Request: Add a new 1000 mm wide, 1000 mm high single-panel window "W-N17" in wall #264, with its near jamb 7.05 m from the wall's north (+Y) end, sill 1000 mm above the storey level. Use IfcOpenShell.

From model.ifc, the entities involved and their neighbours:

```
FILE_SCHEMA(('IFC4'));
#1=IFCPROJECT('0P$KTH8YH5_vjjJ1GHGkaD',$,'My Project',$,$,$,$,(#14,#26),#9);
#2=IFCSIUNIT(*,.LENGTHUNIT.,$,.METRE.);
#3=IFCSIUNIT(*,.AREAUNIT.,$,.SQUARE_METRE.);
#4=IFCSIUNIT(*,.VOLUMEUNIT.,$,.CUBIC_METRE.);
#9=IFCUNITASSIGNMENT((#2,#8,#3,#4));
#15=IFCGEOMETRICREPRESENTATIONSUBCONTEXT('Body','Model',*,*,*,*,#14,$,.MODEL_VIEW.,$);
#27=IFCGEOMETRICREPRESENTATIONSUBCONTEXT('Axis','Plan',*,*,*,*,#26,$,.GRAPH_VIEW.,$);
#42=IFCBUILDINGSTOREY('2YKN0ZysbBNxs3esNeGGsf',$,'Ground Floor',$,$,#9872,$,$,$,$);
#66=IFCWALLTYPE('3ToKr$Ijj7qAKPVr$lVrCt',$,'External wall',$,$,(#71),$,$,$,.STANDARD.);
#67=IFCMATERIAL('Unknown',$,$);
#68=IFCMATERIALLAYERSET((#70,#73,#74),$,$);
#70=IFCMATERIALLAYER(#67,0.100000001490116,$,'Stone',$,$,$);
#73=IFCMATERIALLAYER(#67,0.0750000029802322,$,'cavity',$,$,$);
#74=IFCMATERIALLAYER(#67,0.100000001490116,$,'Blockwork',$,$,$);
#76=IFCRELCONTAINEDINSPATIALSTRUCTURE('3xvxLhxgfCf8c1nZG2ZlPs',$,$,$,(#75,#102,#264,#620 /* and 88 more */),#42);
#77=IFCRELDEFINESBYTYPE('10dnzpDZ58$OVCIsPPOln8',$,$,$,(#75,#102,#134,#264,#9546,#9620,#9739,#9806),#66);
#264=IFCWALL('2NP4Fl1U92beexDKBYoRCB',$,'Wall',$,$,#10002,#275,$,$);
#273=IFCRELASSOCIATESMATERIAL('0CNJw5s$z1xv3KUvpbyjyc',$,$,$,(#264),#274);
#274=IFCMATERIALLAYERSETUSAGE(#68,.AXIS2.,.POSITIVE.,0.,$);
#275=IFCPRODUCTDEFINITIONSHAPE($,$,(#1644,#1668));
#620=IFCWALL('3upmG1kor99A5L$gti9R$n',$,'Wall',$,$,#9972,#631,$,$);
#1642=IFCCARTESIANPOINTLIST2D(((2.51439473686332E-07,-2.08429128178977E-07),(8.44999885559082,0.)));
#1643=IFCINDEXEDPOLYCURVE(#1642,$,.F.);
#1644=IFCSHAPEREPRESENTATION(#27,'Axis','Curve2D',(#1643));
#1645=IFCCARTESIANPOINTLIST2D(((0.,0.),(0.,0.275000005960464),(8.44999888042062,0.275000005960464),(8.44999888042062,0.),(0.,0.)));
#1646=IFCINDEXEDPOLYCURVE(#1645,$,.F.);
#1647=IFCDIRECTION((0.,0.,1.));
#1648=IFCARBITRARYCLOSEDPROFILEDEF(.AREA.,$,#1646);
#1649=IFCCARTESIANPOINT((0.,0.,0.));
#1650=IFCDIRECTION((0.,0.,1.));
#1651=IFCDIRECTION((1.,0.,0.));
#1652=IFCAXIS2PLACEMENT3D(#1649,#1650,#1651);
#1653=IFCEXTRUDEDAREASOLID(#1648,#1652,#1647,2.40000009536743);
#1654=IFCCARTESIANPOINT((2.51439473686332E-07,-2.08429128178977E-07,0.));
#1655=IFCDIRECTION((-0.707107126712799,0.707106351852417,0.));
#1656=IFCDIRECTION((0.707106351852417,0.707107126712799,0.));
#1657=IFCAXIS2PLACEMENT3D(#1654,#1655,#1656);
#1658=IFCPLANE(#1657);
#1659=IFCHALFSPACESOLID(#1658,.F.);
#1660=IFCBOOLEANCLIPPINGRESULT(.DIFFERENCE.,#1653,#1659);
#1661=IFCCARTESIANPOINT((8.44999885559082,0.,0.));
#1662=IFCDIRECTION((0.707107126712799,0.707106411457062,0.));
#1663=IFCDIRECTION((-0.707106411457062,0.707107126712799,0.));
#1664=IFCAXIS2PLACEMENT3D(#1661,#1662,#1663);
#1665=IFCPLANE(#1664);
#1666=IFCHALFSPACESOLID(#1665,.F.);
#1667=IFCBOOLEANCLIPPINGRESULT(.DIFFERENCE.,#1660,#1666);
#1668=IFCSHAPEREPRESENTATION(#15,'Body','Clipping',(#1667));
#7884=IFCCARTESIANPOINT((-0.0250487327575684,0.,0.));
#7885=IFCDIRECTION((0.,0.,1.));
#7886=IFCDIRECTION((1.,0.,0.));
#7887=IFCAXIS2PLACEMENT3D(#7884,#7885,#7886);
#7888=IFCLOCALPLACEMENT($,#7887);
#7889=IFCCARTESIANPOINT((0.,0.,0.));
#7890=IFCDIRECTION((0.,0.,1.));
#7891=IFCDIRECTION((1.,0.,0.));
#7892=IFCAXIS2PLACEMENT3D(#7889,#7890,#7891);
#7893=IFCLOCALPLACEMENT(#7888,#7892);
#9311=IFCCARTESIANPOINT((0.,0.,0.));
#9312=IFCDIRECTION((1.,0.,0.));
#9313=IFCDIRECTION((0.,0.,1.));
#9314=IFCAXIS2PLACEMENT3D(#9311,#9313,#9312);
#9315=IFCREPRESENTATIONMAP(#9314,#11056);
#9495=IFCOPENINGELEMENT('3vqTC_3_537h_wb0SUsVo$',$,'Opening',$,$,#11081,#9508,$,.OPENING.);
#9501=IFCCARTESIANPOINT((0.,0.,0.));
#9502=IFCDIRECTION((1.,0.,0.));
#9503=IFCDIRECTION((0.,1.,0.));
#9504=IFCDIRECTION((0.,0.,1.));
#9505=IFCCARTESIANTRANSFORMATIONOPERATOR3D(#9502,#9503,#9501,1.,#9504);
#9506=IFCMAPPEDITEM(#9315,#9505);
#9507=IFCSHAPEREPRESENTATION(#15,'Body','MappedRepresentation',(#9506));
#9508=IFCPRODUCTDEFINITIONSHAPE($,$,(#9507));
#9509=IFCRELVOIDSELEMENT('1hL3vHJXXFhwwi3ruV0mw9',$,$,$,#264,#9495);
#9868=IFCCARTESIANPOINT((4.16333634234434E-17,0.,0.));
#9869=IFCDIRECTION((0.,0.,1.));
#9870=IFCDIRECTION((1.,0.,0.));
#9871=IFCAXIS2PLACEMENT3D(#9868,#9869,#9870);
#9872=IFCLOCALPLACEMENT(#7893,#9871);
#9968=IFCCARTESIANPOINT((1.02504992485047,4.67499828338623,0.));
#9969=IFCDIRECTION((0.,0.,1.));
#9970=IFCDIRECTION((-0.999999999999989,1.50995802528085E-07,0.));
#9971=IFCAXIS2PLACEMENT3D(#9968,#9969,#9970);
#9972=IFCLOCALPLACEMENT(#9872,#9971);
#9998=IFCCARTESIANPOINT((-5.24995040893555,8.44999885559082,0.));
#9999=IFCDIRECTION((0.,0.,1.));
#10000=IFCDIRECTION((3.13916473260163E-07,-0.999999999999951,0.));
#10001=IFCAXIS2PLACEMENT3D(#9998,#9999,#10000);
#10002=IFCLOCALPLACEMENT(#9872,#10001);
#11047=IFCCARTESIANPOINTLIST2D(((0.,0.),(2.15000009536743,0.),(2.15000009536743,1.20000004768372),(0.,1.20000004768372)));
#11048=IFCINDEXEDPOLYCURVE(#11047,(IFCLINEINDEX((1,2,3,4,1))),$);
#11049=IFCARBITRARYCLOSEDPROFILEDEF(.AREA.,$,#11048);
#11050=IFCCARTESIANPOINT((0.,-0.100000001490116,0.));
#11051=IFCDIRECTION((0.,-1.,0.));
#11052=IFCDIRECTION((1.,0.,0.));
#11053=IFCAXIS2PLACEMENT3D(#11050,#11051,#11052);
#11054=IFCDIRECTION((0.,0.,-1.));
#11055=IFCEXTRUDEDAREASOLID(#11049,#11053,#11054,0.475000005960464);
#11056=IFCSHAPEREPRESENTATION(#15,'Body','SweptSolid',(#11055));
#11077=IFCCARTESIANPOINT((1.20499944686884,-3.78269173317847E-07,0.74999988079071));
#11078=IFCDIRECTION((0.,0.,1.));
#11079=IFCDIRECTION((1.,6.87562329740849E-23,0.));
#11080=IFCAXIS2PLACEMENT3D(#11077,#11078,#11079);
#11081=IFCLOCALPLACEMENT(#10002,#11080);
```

```python
import numpy as np
import ifcopenshell
import ifcopenshell.api.feature
import ifcopenshell.api.geometry
import ifcopenshell.api.root
import ifcopenshell.api.spatial
import ifcopenshell.geom
import ifcopenshell.util.element
import ifcopenshell.util.placement
import ifcopenshell.util.representation
import ifcopenshell.util.shape
import ifcopenshell.util.unit

model = ifcopenshell.open("model.ifc")
unit_scale = ifcopenshell.util.unit.calculate_unit_scale(model)
settings = ifcopenshell.geom.settings()


def volume(element):
    """Net volume in cubic metres, openings subtracted."""
    shape = ifcopenshell.geom.create_shape(settings, element)
    return ifcopenshell.util.shape.get_volume(shape.geometry)


wall = model.by_guid("2NP4Fl1U92beexDKBYoRCB")
storey = ifcopenshell.util.element.get_container(wall, ifc_class="IfcBuildingStorey")
context = ifcopenshell.util.representation.get_context(model, "Model", "Body", "MODEL_VIEW")
before = volume(wall)

width, height, from_end, sill = 1, 1, 7.05, 1  # metres

# The wall runs along its own X axis, and the end named is its -X end.
wall_shape = ifcopenshell.geom.create_shape(settings, wall)
x, y, z = ifcopenshell.util.shape.get_vertices(wall_shape.geometry).T
start = x.min() + from_end
face, thickness = float(y.min()), float(y.max() - y.min())
wall_matrix = ifcopenshell.util.placement.get_local_placement(wall.ObjectPlacement)
level = ifcopenshell.util.placement.get_local_placement(storey.ObjectPlacement)[2, 3]


def in_wall(x, y):
    """Placement at x, y metres in the wall's axes, at sill height."""
    matrix = wall_matrix.copy()
    matrix[:, 3] = wall_matrix @ np.array([x / unit_scale, y / unit_scale, 0.0, 1.0])
    matrix[2, 3] = level + sill / unit_scale
    return matrix


# Opening: a box that overshoots both wall faces by 50 mm.
opening = ifcopenshell.api.root.create_entity(model, ifc_class="IfcOpeningElement", predefined_type="OPENING")
box = ifcopenshell.api.geometry.add_wall_representation(
    model, context=context, length=width, height=height, thickness=thickness + 0.1
)
ifcopenshell.api.geometry.assign_representation(model, product=opening, representation=box)
ifcopenshell.api.geometry.edit_object_placement(model, product=opening, matrix=in_wall(start, face - 0.05), is_si=False)
ifcopenshell.api.feature.add_feature(model, feature=opening, element=wall)

window = ifcopenshell.api.root.create_entity(model, ifc_class="IfcWindow", name="W-N17", predefined_type="WINDOW")
window.OverallWidth, window.OverallHeight = width / unit_scale, height / unit_scale
window.PartitioningType = "SINGLE_PANEL"
body = ifcopenshell.api.geometry.add_window_representation(
    model,
    context=context,
    overall_width=window.OverallWidth,
    overall_height=window.OverallHeight,
    partition_type="SINGLE_PANEL",
)
ifcopenshell.api.geometry.assign_representation(model, product=window, representation=body)
ifcopenshell.api.spatial.assign_container(model, products=[window], relating_structure=storey)
ifcopenshell.api.feature.add_filling(model, opening=opening, element=window)

# Centre the window in the wall's thickness.
ifcopenshell.api.geometry.edit_object_placement(model, product=window, matrix=in_wall(start, face), is_si=False)
window_shape = ifcopenshell.geom.create_shape(settings, window)
depth = ifcopenshell.util.shape.get_vertices(window_shape.geometry)[:, 1]
offset = face + thickness / 2 - (depth.min() + depth.max()) / 2
ifcopenshell.api.geometry.edit_object_placement(model, product=window, matrix=in_wall(start, offset), is_si=False)

after = volume(wall)

print(f"wall volume {before:.3f} -> {after:.3f} m3")

model.write("model_updated.ifc")
```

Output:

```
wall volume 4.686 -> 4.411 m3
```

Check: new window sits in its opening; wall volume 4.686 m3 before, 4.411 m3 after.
